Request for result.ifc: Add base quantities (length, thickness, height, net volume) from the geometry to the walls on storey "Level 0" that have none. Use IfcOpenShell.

First a look at what the model holds.

```python
import ifcopenshell
import ifcopenshell.util.element
import ifcopenshell.util.unit

model = ifcopenshell.open("result.ifc")
print(model.schema)
for unit_type in ("LENGTHUNIT", "AREAUNIT", "VOLUMEUNIT"):
    print(unit_type, ifcopenshell.util.unit.calculate_unit_scale(model, unit_type))
storey = next(s for s in model.by_type("IfcBuildingStorey") if s.Name == "Level 0")
walls = [e for e in ifcopenshell.util.element.get_decomposition(storey) if e.is_a("IfcWall")]
for e in sorted(walls, key=lambda e: e.id()):
    print(e.id(), e.is_a(), e.Name, list(ifcopenshell.util.element.get_psets(e, qtos_only=True)), sep=" | ")
```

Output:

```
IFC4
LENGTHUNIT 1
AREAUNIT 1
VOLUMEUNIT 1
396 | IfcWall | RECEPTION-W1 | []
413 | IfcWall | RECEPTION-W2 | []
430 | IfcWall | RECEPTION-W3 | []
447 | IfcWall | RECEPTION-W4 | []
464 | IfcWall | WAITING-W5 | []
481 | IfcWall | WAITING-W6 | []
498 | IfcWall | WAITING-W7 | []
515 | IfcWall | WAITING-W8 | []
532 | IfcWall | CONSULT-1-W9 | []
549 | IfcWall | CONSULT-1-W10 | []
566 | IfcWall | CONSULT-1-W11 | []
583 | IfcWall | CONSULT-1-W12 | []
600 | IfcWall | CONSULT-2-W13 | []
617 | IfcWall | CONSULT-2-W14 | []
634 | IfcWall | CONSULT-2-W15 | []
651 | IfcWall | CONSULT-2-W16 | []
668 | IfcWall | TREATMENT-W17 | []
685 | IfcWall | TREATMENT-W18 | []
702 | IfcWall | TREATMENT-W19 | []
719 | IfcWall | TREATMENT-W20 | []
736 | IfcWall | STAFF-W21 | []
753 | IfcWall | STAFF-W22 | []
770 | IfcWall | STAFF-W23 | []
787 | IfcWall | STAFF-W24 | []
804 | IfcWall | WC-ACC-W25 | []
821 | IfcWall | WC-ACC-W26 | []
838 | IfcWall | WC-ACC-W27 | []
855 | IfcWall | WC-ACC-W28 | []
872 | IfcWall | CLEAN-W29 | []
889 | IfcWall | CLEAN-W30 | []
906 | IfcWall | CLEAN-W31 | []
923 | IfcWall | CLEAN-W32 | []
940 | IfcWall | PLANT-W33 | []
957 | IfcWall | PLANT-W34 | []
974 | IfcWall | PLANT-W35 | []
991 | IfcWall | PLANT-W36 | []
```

```python
import ifcopenshell
import ifcopenshell.api.pset
import ifcopenshell.geom
import ifcopenshell.util.element
import ifcopenshell.util.shape
import ifcopenshell.util.unit

model = ifcopenshell.open("result.ifc")
unit_scale = ifcopenshell.util.unit.calculate_unit_scale(model)
volume_scale = ifcopenshell.util.unit.calculate_unit_scale(model, "VOLUMEUNIT")
settings = ifcopenshell.geom.settings()

storey = next(s for s in model.by_type("IfcBuildingStorey") if s.Name == "Level 0")
walls = [e for e in ifcopenshell.util.element.get_decomposition(storey) if e.is_a("IfcWall")]

for e in sorted(walls, key=lambda e: e.id()):
    if ifcopenshell.util.element.get_psets(e, qtos_only=True, should_inherit=False):
        continue
    # Geometry comes back in metres, in the element's own axes.
    shape = ifcopenshell.geom.create_shape(settings, e)
    values = {
        "Length": ifcopenshell.util.shape.get_x(shape.geometry) / unit_scale,
        "Width": ifcopenshell.util.shape.get_y(shape.geometry) / unit_scale,
        "Height": ifcopenshell.util.shape.get_z(shape.geometry) / unit_scale,
        "NetVolume": ifcopenshell.util.shape.get_volume(shape.geometry) / volume_scale,
    }
    qto = ifcopenshell.api.pset.add_qto(model, product=e, name="Qto_WallBaseQuantities")
    ifcopenshell.api.pset.edit_qto(model, qto=qto, properties=values)
    print(e.id(), {k: round(v, 3) for k, v in values.items()})

model.write("result_edited.ifc")
```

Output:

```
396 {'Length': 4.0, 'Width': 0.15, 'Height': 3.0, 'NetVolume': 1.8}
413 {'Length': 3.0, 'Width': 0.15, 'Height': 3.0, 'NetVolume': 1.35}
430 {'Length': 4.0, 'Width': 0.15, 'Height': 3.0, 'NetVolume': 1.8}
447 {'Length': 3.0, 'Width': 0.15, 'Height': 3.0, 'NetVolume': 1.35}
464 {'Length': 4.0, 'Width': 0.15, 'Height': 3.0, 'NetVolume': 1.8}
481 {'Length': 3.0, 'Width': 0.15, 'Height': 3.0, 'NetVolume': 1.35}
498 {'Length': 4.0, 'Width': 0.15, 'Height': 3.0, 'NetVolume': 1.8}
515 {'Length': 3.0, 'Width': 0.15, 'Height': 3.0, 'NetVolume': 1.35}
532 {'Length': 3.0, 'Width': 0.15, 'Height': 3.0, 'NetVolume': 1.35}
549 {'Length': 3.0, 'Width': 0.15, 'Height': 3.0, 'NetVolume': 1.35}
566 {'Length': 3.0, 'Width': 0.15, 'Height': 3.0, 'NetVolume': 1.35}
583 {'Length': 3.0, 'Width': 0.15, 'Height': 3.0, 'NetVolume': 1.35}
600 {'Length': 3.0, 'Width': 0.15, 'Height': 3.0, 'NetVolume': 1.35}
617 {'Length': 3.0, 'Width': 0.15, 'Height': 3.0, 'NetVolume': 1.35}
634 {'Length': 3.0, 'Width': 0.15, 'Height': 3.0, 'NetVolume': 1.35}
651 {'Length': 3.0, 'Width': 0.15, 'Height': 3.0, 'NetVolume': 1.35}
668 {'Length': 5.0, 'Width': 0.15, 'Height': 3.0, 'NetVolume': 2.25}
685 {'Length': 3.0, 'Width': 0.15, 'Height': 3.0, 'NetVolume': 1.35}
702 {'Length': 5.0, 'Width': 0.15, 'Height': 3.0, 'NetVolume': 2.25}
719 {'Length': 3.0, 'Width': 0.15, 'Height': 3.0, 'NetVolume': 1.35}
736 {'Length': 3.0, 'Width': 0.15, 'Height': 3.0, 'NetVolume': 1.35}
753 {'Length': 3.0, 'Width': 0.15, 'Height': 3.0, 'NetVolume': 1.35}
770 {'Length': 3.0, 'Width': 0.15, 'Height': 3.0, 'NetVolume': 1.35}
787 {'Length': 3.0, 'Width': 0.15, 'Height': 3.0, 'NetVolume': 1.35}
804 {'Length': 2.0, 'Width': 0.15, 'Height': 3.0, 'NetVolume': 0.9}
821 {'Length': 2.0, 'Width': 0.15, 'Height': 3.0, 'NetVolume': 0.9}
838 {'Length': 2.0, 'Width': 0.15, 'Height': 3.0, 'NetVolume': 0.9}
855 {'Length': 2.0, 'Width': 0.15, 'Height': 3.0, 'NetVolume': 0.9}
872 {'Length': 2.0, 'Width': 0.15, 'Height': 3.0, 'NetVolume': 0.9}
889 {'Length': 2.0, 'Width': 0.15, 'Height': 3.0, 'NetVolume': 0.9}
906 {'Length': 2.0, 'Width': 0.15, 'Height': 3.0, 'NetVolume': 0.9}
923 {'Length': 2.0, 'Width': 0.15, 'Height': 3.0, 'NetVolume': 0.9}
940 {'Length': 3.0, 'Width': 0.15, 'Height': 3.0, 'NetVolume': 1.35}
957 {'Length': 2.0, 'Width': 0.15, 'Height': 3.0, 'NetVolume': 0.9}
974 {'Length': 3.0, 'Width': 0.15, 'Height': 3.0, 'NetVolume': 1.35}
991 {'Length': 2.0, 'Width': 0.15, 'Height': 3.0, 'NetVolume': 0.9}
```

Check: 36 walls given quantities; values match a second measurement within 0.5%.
